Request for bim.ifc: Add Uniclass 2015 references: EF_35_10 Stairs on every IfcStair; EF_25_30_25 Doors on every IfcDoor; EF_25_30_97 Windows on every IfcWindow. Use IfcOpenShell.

First a look at what the model holds.

```python
import ifcopenshell

model = ifcopenshell.open("bim.ifc")
print(model.schema)
print("classifications:", [c.Name for c in model.by_type("IfcClassification")])
for ifc_class in ("IfcDoor", "IfcRoof", "IfcStair", "IfcWall", "IfcWindow"):
    print(ifc_class, len(model.by_type(ifc_class)))
```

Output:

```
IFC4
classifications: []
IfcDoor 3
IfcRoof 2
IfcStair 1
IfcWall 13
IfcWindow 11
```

```python
import ifcopenshell
import ifcopenshell.api.classification

model = ifcopenshell.open("bim.ifc")

system = ifcopenshell.api.classification.add_classification(model, classification="Uniclass 2015")

codes = {
    "IfcStair": ("EF_35_10", "Stairs"),
    "IfcDoor": ("EF_25_30_25", "Doors"),
    "IfcWindow": ("EF_25_30_97", "Windows"),
}
for ifc_class, (code, name) in codes.items():
    products = model.by_type(ifc_class)
    ifcopenshell.api.classification.add_reference(
        model, products=products, classification=system, identification=code, name=name
    )
    print(code, len(products))

model.write("bim_rev.ifc")
```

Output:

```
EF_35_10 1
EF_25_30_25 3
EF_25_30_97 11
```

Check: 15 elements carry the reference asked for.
